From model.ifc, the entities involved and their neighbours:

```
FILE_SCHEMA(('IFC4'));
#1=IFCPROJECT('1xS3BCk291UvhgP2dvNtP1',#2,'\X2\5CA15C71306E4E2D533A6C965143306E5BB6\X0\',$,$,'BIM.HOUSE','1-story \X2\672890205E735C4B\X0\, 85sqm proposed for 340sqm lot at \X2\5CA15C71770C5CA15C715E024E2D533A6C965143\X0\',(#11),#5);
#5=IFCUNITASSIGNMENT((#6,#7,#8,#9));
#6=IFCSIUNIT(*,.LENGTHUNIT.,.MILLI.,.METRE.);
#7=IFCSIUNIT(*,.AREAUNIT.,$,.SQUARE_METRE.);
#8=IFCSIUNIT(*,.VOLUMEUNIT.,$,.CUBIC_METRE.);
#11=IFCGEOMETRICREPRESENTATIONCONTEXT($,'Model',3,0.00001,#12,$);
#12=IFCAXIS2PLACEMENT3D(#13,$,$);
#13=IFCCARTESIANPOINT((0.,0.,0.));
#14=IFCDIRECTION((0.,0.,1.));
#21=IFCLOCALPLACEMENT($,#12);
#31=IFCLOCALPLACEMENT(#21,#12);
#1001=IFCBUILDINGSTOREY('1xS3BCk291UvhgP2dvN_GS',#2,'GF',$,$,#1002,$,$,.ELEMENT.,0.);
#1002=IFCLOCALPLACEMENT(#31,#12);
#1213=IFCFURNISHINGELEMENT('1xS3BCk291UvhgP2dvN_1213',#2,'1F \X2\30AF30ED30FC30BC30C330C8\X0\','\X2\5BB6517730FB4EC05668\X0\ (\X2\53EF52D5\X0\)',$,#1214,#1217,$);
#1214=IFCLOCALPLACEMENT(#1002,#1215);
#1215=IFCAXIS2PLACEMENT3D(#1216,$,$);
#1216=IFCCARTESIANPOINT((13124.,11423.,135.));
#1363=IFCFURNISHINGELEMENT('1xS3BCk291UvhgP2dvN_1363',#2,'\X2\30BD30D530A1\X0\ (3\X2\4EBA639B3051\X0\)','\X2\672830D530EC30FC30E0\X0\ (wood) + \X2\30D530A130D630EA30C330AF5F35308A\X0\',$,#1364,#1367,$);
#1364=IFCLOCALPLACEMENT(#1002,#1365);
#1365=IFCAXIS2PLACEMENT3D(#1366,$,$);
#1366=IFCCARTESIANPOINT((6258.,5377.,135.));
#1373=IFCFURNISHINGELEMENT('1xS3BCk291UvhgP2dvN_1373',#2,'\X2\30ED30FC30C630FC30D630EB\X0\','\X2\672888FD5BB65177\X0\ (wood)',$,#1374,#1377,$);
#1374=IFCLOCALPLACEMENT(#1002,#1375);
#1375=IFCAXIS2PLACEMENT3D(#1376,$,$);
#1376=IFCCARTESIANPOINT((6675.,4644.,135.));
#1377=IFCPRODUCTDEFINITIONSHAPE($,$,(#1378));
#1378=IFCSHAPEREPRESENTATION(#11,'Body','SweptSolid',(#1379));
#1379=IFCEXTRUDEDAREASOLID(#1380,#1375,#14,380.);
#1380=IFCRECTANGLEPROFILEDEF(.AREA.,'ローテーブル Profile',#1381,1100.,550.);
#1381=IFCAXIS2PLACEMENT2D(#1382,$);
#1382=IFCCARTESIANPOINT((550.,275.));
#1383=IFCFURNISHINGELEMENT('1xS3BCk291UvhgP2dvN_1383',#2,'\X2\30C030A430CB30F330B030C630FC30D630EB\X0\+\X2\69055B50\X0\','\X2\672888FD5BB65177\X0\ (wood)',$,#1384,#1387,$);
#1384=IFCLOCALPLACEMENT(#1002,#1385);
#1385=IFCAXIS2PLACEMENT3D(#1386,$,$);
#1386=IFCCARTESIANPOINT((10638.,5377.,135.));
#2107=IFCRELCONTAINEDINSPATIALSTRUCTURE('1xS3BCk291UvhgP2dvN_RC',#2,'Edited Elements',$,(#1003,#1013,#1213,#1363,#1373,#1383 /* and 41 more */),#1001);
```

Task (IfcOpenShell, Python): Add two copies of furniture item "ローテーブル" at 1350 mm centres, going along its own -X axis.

```python
import ifcopenshell
import ifcopenshell.api.geometry
import ifcopenshell.api.root
import ifcopenshell.util.element
import ifcopenshell.util.placement

model = ifcopenshell.open("model.ifc")


def reuse_history(source, copy):
    """copy_class also copies each property set's owner history, people and application; keep the originals."""
    for rel in copy.IsDefinedBy:
        if rel.is_a("IfcRelDefinesByProperties") and (history := rel.RelatingPropertyDefinition.OwnerHistory):
            rel.RelatingPropertyDefinition.OwnerHistory = source.OwnerHistory
            ifcopenshell.util.element.remove_deep2(model, history)


source = model.by_guid("1xS3BCk291UvhgP2dvN_1373")
base = ifcopenshell.util.placement.get_local_placement(source.ObjectPlacement)
step = -base[:3, 0] * 1350.0

for i in range(1, 3):
    copy = ifcopenshell.api.root.copy_class(model, product=source)
    copy.Representation = ifcopenshell.util.element.copy_deep(
        model, source.Representation, exclude=["IfcGeometricRepresentationContext", "IfcRepresentationMap"]
    )
    reuse_history(source, copy)
    matrix = base.copy()
    matrix[:3, 3] += i * step
    print("added at", matrix[:3, 3].round(3) + 0.0)
    ifcopenshell.api.geometry.edit_object_placement(model, product=copy, matrix=matrix, is_si=False)

model.write("model_updated.ifc")
```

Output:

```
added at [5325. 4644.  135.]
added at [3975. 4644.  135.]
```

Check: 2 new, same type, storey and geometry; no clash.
